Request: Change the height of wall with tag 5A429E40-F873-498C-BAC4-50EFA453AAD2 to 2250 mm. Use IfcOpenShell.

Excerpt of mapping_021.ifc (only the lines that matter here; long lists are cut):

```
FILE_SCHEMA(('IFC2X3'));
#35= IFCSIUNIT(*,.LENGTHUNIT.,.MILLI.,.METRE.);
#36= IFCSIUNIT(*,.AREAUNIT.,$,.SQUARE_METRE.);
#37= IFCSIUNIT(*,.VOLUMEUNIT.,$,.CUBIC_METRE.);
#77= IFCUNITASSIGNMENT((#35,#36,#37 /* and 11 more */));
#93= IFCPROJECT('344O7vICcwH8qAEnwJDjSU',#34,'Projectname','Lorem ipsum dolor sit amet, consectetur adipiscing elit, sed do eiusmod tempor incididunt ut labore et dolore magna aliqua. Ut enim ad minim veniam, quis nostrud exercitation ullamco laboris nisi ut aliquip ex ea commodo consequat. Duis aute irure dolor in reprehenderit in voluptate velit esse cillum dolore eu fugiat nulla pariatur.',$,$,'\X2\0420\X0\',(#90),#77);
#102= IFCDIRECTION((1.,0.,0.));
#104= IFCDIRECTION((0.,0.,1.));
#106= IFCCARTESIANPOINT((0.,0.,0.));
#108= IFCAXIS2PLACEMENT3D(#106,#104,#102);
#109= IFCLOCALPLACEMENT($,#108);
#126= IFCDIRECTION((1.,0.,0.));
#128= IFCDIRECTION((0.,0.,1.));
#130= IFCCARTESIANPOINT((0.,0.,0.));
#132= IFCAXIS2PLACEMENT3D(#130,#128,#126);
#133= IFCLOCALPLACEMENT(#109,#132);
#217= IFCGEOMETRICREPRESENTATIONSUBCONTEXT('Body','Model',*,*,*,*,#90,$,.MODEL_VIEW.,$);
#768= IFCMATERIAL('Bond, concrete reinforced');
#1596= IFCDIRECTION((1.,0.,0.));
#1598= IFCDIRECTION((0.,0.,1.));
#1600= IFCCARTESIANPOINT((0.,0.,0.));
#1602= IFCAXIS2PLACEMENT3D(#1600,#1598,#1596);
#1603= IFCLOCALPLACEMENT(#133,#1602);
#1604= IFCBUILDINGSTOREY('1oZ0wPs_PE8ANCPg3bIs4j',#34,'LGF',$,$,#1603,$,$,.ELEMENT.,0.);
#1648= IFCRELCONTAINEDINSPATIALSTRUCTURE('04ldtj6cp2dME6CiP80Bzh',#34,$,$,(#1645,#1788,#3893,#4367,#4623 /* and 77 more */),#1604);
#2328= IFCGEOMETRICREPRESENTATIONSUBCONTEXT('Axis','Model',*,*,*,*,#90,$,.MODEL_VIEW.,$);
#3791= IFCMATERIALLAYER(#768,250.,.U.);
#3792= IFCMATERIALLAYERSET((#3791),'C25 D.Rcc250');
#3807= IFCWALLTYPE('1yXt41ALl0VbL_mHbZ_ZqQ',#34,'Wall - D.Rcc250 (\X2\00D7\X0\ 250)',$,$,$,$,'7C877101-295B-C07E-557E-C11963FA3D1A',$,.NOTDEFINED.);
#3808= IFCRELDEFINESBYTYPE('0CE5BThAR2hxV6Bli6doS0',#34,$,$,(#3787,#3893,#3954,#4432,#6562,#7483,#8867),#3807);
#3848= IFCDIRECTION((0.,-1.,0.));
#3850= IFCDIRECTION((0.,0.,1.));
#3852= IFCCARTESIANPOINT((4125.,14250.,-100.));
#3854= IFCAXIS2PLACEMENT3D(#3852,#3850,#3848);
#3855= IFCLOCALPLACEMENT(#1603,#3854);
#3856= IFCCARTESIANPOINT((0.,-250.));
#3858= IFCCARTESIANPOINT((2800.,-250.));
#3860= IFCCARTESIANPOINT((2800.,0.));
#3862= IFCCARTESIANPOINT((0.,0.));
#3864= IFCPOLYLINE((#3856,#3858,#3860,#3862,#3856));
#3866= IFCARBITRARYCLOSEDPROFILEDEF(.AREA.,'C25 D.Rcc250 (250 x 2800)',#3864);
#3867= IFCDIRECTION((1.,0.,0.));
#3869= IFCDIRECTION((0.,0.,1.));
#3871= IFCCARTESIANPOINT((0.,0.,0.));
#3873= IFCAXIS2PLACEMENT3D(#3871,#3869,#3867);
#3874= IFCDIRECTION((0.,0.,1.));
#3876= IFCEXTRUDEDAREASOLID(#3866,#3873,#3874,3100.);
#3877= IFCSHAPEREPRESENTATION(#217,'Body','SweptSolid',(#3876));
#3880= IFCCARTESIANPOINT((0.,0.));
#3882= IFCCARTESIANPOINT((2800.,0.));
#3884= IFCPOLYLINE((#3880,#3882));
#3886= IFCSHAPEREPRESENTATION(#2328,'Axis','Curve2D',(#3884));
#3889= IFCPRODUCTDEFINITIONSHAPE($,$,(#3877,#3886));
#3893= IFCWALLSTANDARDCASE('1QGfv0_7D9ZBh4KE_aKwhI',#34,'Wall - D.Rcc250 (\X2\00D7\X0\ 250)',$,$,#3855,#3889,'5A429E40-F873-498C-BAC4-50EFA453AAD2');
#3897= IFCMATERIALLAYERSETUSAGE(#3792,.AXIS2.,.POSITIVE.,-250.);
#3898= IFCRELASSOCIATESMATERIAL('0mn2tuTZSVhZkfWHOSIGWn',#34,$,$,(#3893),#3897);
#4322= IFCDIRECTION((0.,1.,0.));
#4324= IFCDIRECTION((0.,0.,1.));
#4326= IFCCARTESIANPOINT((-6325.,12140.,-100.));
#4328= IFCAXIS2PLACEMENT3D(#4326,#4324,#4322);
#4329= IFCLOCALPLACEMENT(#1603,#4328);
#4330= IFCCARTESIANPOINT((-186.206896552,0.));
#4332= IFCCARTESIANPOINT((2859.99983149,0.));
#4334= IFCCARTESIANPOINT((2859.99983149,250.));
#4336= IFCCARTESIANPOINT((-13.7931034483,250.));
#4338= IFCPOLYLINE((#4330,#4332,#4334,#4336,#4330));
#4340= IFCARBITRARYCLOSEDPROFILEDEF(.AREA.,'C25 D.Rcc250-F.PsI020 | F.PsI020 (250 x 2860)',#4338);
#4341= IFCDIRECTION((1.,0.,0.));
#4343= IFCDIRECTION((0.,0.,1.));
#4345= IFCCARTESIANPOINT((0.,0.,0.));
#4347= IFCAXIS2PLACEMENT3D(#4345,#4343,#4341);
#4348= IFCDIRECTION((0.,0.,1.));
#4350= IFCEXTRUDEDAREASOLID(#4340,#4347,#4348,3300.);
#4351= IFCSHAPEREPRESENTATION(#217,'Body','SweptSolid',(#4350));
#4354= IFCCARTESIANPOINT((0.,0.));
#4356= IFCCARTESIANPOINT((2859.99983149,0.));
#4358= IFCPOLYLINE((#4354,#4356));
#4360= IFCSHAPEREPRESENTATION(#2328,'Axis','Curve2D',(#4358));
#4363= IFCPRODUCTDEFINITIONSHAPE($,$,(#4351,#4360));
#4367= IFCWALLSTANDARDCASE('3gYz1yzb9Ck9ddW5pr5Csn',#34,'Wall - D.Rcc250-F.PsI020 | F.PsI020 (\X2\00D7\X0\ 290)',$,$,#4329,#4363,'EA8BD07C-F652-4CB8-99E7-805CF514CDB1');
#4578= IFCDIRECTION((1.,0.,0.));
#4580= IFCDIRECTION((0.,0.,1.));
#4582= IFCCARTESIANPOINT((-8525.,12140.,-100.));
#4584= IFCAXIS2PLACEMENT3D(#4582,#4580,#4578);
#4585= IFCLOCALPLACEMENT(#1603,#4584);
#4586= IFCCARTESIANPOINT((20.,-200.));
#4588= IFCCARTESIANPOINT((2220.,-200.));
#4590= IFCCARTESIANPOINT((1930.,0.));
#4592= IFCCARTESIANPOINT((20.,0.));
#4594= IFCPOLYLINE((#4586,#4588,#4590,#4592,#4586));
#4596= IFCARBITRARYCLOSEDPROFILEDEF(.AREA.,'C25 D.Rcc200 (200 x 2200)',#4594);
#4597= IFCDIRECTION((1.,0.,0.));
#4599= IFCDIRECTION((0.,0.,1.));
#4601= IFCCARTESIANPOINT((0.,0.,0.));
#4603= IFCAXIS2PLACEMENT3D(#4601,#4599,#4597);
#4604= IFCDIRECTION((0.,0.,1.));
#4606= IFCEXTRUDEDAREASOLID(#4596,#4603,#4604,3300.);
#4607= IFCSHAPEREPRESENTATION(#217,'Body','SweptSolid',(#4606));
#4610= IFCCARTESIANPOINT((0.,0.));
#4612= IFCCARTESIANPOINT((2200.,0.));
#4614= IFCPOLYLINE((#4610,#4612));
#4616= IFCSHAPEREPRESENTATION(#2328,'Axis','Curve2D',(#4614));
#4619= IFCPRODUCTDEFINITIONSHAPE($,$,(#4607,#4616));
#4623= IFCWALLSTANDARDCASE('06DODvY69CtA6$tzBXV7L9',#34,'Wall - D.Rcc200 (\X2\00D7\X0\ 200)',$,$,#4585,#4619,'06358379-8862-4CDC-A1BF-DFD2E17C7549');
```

```python
import ifcopenshell
import ifcopenshell.geom
import ifcopenshell.util.representation
import ifcopenshell.util.shape
import ifcopenshell.util.unit

model = ifcopenshell.open("mapping_021.ifc")
unit_scale = ifcopenshell.util.unit.calculate_unit_scale(model)
settings = ifcopenshell.geom.settings()


def volume(element):
    """Net volume in cubic metres, openings subtracted."""
    shape = ifcopenshell.geom.create_shape(settings, element)
    return ifcopenshell.util.shape.get_volume(shape.geometry)


wall = model.by_guid("1QGfv0_7D9ZBh4KE_aKwhI")
before = volume(wall)

body = ifcopenshell.util.representation.get_representation(wall, "Model", "Body")
solid = body.Items[0]
old_height = solid.Depth
solid.Depth = 2.25 / unit_scale
after = volume(wall)

print(f"height {old_height:g} -> {solid.Depth:g}, volume {before:.3f} -> {after:.3f} m3")

model.write("mapping_021-out.ifc")
```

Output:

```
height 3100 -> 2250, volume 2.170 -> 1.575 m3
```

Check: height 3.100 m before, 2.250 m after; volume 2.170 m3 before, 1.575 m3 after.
